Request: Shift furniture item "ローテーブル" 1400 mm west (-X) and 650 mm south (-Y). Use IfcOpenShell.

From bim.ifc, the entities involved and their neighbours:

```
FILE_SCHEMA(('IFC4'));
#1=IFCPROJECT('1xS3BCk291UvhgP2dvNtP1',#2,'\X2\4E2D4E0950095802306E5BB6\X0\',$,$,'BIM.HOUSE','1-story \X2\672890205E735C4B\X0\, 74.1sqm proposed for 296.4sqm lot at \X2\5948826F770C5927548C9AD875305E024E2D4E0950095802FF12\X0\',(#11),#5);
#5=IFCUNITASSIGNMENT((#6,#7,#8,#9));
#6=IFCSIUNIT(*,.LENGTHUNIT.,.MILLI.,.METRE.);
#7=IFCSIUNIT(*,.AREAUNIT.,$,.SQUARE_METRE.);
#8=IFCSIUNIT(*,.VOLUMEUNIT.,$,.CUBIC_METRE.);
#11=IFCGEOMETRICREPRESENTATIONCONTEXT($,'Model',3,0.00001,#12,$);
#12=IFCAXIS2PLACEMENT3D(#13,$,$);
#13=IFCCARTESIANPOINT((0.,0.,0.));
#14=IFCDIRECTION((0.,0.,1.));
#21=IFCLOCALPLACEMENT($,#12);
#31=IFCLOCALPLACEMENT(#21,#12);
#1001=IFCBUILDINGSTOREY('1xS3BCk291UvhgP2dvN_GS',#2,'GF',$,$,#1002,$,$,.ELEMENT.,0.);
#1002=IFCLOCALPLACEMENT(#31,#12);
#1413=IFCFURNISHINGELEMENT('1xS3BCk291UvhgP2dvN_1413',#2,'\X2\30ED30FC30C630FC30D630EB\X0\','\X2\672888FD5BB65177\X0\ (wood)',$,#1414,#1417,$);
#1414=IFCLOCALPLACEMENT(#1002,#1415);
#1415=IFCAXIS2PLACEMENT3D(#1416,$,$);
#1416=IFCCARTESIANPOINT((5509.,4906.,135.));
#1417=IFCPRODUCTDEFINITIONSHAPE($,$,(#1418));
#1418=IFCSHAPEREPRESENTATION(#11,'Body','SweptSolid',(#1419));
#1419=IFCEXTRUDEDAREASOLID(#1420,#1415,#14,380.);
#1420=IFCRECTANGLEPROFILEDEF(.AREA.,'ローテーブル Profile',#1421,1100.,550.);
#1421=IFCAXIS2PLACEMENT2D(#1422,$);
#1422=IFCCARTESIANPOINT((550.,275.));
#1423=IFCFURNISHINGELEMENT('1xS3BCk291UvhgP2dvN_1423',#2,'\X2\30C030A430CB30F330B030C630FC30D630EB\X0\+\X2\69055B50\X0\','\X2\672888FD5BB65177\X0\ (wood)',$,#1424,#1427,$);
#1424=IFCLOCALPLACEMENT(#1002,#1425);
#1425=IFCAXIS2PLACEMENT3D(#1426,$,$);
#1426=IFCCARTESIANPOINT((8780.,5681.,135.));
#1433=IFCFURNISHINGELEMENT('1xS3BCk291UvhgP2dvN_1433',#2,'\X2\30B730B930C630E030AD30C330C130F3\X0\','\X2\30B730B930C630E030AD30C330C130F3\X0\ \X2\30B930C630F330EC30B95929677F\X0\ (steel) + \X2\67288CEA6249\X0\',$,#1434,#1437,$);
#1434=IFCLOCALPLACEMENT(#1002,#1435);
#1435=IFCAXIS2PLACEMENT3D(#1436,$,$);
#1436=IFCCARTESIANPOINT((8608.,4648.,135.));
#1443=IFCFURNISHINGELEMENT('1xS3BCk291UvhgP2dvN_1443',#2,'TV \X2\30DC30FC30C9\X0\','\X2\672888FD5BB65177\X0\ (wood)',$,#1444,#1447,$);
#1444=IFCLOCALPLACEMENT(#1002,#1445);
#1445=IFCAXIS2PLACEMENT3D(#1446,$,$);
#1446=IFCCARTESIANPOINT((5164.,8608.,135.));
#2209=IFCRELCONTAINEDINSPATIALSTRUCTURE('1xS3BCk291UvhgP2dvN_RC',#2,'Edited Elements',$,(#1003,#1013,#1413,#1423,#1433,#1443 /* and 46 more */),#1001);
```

```python
import ifcopenshell
import ifcopenshell.api.geometry
import ifcopenshell.util.placement
import ifcopenshell.util.unit

model = ifcopenshell.open("bim.ifc")
unit_scale = ifcopenshell.util.unit.calculate_unit_scale(model)

item = model.by_guid("1xS3BCk291UvhgP2dvN_1413")
matrix = ifcopenshell.util.placement.get_local_placement(item.ObjectPlacement)
matrix[0, 3] -= 1.4 / unit_scale
matrix[1, 3] -= 0.65 / unit_scale
ifcopenshell.api.geometry.edit_object_placement(model, product=item, matrix=matrix, is_si=False)

print(ifcopenshell.util.placement.get_local_placement(item.ObjectPlacement).round(3) + 0.0)

model.write("bim_rev.ifc")
```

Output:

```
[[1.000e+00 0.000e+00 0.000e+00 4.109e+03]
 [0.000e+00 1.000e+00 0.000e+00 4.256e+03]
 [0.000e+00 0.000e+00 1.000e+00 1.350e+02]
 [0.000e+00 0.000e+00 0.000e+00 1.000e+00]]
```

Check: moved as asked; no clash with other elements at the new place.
